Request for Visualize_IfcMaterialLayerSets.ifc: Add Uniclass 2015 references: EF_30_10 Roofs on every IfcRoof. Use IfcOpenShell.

First a look at what the model holds.

```python
import ifcopenshell

model = ifcopenshell.open("Visualize_IfcMaterialLayerSets.ifc")
print(model.schema)
print("classifications:", [c.Name for c in model.by_type("IfcClassification")])
for ifc_class in ("IfcDoor", "IfcRoof", "IfcStair", "IfcWall", "IfcWindow"):
    print(ifc_class, len(model.by_type(ifc_class)))
```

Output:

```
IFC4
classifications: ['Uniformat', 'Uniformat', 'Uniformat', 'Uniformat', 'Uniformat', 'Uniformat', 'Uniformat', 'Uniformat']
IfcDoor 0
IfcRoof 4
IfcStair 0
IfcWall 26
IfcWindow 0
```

```python
import ifcopenshell
import ifcopenshell.api.classification

model = ifcopenshell.open("Visualize_IfcMaterialLayerSets.ifc")

system = ifcopenshell.api.classification.add_classification(model, classification="Uniclass 2015")

codes = {
    "IfcRoof": ("EF_30_10", "Roofs"),
}
for ifc_class, (code, name) in codes.items():
    products = model.by_type(ifc_class)
    ifcopenshell.api.classification.add_reference(
        model, products=products, classification=system, identification=code, name=name
    )
    print(code, len(products))

model.write("Visualize_IfcMaterialLayerSets_rev.ifc")
```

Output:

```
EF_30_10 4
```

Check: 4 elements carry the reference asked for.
